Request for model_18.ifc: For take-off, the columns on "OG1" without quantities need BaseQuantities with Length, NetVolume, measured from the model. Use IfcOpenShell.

First a look at what the model holds.

```python
import ifcopenshell
import ifcopenshell.util.element
import ifcopenshell.util.unit

model = ifcopenshell.open("model_18.ifc")
print(model.schema)
for unit_type in ("LENGTHUNIT", "AREAUNIT", "VOLUMEUNIT"):
    print(unit_type, ifcopenshell.util.unit.calculate_unit_scale(model, unit_type))
storey = next(s for s in model.by_type("IfcBuildingStorey") if s.Name == "OG1")
columns = [e for e in ifcopenshell.util.element.get_decomposition(storey) if e.is_a("IfcColumn")]
for e in sorted(columns, key=lambda e: e.id()):
    print(e.id(), e.is_a(), e.Name, list(ifcopenshell.util.element.get_psets(e, qtos_only=True)), sep=" | ")
```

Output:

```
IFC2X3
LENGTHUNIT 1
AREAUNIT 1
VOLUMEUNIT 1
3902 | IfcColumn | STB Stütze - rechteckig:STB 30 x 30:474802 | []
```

```python
import ifcopenshell
import ifcopenshell.api.pset
import ifcopenshell.geom
import ifcopenshell.util.element
import ifcopenshell.util.shape
import ifcopenshell.util.unit

model = ifcopenshell.open("model_18.ifc")
unit_scale = ifcopenshell.util.unit.calculate_unit_scale(model)
volume_scale = ifcopenshell.util.unit.calculate_unit_scale(model, "VOLUMEUNIT")
settings = ifcopenshell.geom.settings()

storey = next(s for s in model.by_type("IfcBuildingStorey") if s.Name == "OG1")
columns = [e for e in ifcopenshell.util.element.get_decomposition(storey) if e.is_a("IfcColumn")]

for e in sorted(columns, key=lambda e: e.id()):
    if ifcopenshell.util.element.get_psets(e, qtos_only=True, should_inherit=False):
        continue
    # Geometry comes back in metres, in the element's own axes.
    shape = ifcopenshell.geom.create_shape(settings, e)
    values = {
        "Length": ifcopenshell.util.shape.get_z(shape.geometry) / unit_scale,
        "NetVolume": ifcopenshell.util.shape.get_volume(shape.geometry) / volume_scale,
    }
    qto = ifcopenshell.api.pset.add_qto(model, product=e, name="BaseQuantities")
    ifcopenshell.api.pset.edit_qto(model, qto=qto, properties=values)
    print(e.id(), {k: round(v, 3) for k, v in values.items()})

model.write("model_18_rev.ifc")
```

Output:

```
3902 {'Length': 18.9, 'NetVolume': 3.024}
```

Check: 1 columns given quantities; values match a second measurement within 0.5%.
